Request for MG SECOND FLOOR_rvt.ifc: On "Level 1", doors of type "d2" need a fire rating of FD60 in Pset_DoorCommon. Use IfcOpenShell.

First a look at what the model holds.

```python
import ifcopenshell
import ifcopenshell.util.element

model = ifcopenshell.open("MG SECOND FLOOR_rvt.ifc")
print(model.schema)
storey = next(s for s in model.by_type("IfcBuildingStorey") if s.Name == "Level 1")
doors = [e for e in ifcopenshell.util.element.get_decomposition(storey) if e.is_a("IfcDoor")]
seen = {}
for e in doors:
    element_type = ifcopenshell.util.element.get_type(e)
    key = (element_type.Name if element_type != e and element_type else None, ifcopenshell.util.element.get_pset(e, "Pset_DoorCommon", "FireRating"))
    seen[key] = seen.get(key, 0) + 1
for (name, value), count in sorted(seen.items(), key=str):
    print(count, "x", name, "|", value)
```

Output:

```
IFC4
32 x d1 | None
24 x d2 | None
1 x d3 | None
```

```python
import ifcopenshell
import ifcopenshell.api.pset
import ifcopenshell.util.element

model = ifcopenshell.open("MG SECOND FLOOR_rvt.ifc")

storey = next(s for s in model.by_type("IfcBuildingStorey") if s.Name == "Level 1")
doors = [e for e in ifcopenshell.util.element.get_decomposition(storey) if e.is_a("IfcDoor")]

count = 0
for e in doors:
    element_type = ifcopenshell.util.element.get_type(e)
    if element_type in (None, e) or element_type.Name != "d2":
        continue
    # add_pset returns the element's existing set when there is one.
    pset = ifcopenshell.api.pset.add_pset(model, product=e, name="Pset_DoorCommon")
    ifcopenshell.api.pset.edit_pset(model, pset=pset, properties={"FireRating": "FD60"})
    count += 1

print(count, "doors updated")

model.write("MG SECOND FLOOR_rvt-out.ifc")
```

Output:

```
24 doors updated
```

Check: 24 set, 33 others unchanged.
